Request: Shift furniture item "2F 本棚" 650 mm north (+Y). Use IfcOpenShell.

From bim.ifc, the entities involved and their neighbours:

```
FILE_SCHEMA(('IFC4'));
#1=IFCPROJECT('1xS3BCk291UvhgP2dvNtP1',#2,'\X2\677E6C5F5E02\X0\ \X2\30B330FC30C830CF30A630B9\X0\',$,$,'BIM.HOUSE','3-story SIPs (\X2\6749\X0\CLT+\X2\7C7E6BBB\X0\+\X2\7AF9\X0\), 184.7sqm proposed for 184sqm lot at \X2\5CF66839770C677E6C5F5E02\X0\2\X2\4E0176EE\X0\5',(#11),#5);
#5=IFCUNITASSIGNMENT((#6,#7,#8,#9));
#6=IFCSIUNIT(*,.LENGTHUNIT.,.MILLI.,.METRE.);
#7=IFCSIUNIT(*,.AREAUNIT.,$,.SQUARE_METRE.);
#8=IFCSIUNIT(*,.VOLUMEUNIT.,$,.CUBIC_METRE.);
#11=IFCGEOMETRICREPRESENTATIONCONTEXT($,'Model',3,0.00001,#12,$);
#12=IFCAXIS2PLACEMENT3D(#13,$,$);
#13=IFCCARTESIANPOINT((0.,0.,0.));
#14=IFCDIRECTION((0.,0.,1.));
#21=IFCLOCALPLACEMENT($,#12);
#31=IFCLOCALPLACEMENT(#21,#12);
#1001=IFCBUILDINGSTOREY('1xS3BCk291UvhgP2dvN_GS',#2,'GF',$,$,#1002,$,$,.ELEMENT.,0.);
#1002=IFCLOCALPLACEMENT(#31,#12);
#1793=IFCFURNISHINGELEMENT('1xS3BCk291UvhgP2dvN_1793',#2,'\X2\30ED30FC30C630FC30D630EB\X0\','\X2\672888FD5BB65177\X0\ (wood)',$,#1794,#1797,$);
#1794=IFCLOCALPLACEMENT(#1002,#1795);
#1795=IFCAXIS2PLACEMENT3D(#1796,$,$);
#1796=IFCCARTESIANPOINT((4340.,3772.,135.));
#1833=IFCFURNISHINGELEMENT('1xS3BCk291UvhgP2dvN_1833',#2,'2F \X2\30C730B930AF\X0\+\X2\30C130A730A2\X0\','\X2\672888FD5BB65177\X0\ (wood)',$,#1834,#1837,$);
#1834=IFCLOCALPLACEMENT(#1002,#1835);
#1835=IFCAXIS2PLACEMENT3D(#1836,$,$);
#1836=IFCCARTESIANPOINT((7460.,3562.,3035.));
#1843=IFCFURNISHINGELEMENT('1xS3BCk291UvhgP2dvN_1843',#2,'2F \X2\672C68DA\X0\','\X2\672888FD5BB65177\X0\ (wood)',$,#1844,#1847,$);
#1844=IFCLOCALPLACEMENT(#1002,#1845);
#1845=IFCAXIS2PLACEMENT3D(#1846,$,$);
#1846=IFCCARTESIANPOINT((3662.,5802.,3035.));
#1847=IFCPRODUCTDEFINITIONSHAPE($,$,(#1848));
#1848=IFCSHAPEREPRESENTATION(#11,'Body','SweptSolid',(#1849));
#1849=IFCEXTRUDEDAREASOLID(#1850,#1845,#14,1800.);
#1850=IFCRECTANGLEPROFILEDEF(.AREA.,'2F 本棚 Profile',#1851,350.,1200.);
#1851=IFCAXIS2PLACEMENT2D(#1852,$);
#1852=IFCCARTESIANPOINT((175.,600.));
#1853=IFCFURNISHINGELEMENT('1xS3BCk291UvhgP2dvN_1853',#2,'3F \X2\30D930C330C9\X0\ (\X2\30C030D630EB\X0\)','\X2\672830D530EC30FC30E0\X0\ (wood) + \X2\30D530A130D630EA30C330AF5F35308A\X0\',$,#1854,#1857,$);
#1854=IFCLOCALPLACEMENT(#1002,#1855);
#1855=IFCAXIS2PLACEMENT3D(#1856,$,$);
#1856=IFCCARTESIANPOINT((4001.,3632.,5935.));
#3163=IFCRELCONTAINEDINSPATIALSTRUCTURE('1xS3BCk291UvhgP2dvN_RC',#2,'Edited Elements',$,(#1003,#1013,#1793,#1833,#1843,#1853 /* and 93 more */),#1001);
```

```python
import ifcopenshell
import ifcopenshell.api.geometry
import ifcopenshell.util.placement

model = ifcopenshell.open("bim.ifc")

item = model.by_guid("1xS3BCk291UvhgP2dvN_1843")
matrix = ifcopenshell.util.placement.get_local_placement(item.ObjectPlacement)
matrix[1, 3] += 650.0
ifcopenshell.api.geometry.edit_object_placement(model, product=item, matrix=matrix, is_si=False)

print(ifcopenshell.util.placement.get_local_placement(item.ObjectPlacement).round(3) + 0.0)

model.write("bim_edited.ifc")
```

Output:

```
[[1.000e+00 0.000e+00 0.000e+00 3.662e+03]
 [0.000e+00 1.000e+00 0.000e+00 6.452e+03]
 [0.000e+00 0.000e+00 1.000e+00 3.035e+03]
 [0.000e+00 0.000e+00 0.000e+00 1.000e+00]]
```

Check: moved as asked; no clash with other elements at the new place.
